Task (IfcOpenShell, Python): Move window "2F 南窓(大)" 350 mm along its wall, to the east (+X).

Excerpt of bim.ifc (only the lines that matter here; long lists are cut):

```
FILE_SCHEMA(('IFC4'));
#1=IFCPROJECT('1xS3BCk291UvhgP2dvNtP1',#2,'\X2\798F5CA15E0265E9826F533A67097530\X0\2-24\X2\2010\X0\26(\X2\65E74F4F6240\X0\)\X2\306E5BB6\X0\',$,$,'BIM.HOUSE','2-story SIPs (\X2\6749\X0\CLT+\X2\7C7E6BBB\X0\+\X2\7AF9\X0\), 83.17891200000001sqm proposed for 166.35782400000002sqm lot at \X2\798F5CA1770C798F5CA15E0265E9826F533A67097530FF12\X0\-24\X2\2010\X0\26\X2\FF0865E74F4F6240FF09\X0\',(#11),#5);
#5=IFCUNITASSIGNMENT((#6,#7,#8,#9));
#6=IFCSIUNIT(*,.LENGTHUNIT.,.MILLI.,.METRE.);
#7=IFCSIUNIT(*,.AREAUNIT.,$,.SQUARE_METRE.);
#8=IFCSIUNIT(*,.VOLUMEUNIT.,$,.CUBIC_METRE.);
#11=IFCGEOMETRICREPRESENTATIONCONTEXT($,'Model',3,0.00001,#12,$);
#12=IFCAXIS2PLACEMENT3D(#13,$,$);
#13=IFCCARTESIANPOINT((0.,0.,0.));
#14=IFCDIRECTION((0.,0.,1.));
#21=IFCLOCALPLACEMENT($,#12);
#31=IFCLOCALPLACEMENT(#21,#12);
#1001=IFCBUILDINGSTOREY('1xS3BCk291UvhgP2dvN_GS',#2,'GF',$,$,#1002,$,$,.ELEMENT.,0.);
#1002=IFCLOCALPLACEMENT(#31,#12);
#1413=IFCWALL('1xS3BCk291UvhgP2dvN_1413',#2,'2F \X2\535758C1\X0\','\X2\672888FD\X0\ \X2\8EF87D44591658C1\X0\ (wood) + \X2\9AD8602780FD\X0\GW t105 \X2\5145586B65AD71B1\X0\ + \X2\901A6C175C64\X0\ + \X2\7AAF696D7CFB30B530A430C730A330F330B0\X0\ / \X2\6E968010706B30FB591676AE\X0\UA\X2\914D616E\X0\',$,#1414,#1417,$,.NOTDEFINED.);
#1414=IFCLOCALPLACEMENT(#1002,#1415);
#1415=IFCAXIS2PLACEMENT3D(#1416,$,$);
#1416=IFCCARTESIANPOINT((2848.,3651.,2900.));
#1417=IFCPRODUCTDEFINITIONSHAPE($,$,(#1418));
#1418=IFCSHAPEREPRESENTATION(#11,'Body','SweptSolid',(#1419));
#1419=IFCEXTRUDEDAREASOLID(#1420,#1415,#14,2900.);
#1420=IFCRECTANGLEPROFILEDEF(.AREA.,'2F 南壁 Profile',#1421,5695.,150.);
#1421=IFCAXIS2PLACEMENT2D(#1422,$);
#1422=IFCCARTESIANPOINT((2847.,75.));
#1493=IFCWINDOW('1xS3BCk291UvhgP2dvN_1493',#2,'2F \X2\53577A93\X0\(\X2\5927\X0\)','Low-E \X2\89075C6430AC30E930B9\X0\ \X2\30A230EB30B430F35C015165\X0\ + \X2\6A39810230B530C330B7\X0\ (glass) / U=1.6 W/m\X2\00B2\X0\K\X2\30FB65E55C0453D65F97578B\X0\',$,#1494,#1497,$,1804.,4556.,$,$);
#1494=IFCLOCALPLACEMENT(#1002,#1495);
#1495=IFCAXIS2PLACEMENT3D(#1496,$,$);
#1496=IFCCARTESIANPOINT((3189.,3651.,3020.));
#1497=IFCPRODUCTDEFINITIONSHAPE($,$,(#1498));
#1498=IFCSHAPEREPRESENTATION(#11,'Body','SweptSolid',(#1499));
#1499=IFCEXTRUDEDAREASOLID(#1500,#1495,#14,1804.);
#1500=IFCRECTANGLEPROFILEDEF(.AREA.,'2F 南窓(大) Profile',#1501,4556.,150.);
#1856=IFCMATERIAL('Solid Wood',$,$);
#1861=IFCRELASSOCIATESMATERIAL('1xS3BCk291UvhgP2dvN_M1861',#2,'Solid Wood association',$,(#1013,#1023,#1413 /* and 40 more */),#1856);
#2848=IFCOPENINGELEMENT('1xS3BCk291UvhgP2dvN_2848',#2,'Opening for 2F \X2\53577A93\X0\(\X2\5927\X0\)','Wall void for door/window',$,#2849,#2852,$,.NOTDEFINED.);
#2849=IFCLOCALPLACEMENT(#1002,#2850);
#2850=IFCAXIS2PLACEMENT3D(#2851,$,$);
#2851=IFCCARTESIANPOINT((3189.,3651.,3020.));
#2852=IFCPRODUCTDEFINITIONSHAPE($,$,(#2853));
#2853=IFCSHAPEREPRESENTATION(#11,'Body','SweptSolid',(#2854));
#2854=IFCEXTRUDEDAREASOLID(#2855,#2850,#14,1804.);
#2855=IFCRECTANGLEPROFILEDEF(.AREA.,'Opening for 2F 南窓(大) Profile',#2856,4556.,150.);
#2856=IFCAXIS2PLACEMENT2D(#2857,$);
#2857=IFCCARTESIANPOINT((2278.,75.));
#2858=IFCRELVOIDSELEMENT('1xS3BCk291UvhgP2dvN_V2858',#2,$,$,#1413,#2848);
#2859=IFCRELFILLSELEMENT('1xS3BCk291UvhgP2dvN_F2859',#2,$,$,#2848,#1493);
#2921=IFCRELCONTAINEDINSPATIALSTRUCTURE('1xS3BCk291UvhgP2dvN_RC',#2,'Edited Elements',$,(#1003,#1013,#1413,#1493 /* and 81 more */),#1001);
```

```python
import ifcopenshell
import ifcopenshell.api.geometry
import ifcopenshell.util.placement

model = ifcopenshell.open("bim.ifc")

window = model.by_id(1493)
opening = window.FillsVoids[0].RelatingOpeningElement
wall = opening.VoidsElements[0].RelatingBuildingElement

wall_matrix = ifcopenshell.util.placement.get_local_placement(wall.ObjectPlacement)
shift = wall_matrix[:3, 0] * 350.0
before = ifcopenshell.util.placement.get_local_placement(window.ObjectPlacement)[:3, 3].copy()

# The window is not placed relative to its opening, so move both.
for product in (opening, window):
    matrix = ifcopenshell.util.placement.get_local_placement(product.ObjectPlacement)
    matrix[:3, 3] += shift
    ifcopenshell.api.geometry.edit_object_placement(model, product=product, matrix=matrix, is_si=False)

after = ifcopenshell.util.placement.get_local_placement(window.ObjectPlacement)[:3, 3]
print("window moved by", (after - before).round(3) + 0.0)

model.write("bim_edited.ifc")
```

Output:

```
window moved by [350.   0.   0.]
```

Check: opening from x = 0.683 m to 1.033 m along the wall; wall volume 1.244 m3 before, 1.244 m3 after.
